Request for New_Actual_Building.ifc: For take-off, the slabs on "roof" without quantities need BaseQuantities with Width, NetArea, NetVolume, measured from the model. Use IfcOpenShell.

First a look at what the model holds.

```python
import ifcopenshell
import ifcopenshell.util.element
import ifcopenshell.util.unit

model = ifcopenshell.open("New_Actual_Building.ifc")
print(model.schema)
for unit_type in ("LENGTHUNIT", "AREAUNIT", "VOLUMEUNIT"):
    print(unit_type, ifcopenshell.util.unit.calculate_unit_scale(model, unit_type))
storey = next(s for s in model.by_type("IfcBuildingStorey") if s.Name == "roof")
slabs = [e for e in ifcopenshell.util.element.get_decomposition(storey) if e.is_a("IfcSlab")]
for e in sorted(slabs, key=lambda e: e.id()):
    print(e.id(), e.is_a(), e.Name, list(ifcopenshell.util.element.get_psets(e, qtos_only=True)), sep=" | ")
```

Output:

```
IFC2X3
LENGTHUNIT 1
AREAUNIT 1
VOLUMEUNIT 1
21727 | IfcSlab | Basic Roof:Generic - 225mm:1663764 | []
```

```python
import ifcopenshell
import ifcopenshell.api.pset
import ifcopenshell.geom
import ifcopenshell.util.element
import ifcopenshell.util.shape
import ifcopenshell.util.unit

model = ifcopenshell.open("New_Actual_Building.ifc")
unit_scale = ifcopenshell.util.unit.calculate_unit_scale(model)
area_scale = ifcopenshell.util.unit.calculate_unit_scale(model, "AREAUNIT")
volume_scale = ifcopenshell.util.unit.calculate_unit_scale(model, "VOLUMEUNIT")
settings = ifcopenshell.geom.settings()

storey = next(s for s in model.by_type("IfcBuildingStorey") if s.Name == "roof")
slabs = [e for e in ifcopenshell.util.element.get_decomposition(storey) if e.is_a("IfcSlab")]

for e in sorted(slabs, key=lambda e: e.id()):
    if ifcopenshell.util.element.get_psets(e, qtos_only=True, should_inherit=False):
        continue
    # Geometry comes back in metres, in the element's own axes.
    shape = ifcopenshell.geom.create_shape(settings, e)
    values = {
        "Width": ifcopenshell.util.shape.get_z(shape.geometry) / unit_scale,
        "NetArea": ifcopenshell.util.shape.get_footprint_area(shape.geometry) / area_scale,
        "NetVolume": ifcopenshell.util.shape.get_volume(shape.geometry) / volume_scale,
    }
    qto = ifcopenshell.api.pset.add_qto(model, product=e, name="BaseQuantities")
    ifcopenshell.api.pset.edit_qto(model, qto=qto, properties=values)
    print(e.id(), {k: round(v, 3) for k, v in values.items()})

model.write("New_Actual_Building_v2.ifc")
```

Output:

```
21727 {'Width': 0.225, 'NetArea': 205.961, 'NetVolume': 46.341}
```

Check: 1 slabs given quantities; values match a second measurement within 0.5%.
